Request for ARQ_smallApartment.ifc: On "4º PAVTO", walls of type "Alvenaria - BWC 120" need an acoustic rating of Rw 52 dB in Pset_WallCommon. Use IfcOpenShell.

First a look at what the model holds.

```python
import ifcopenshell
import ifcopenshell.util.element

model = ifcopenshell.open("ARQ_smallApartment.ifc")
print(model.schema)
storey = next(s for s in model.by_type("IfcBuildingStorey") if s.Name == "4º PAVTO")
walls = [e for e in ifcopenshell.util.element.get_decomposition(storey) if e.is_a("IfcWall")]
seen = {}
for e in walls:
    element_type = ifcopenshell.util.element.get_type(e)
    key = (element_type.Name if element_type != e and element_type else None, ifcopenshell.util.element.get_pset(e, "Pset_WallCommon", "AcousticRating"))
    seen[key] = seen.get(key, 0) + 1
for (name, value), count in sorted(seen.items(), key=str):
    print(count, "x", name, "|", value)
```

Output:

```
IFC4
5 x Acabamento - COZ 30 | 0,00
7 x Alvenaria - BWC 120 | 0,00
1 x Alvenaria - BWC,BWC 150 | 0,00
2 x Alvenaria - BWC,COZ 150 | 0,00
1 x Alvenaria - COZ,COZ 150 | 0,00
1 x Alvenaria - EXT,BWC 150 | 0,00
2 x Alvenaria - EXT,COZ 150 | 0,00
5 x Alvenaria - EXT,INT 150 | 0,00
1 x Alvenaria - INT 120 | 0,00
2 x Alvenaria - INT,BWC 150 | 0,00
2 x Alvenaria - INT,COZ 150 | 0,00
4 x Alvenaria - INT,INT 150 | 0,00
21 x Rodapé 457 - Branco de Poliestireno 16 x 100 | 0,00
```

```python
import ifcopenshell
import ifcopenshell.api.pset
import ifcopenshell.util.element

model = ifcopenshell.open("ARQ_smallApartment.ifc")

storey = next(s for s in model.by_type("IfcBuildingStorey") if s.Name == "4º PAVTO")
walls = [e for e in ifcopenshell.util.element.get_decomposition(storey) if e.is_a("IfcWall")]

count = 0
for e in walls:
    element_type = ifcopenshell.util.element.get_type(e)
    if element_type in (None, e) or element_type.Name != "Alvenaria - BWC 120":
        continue
    # add_pset returns the element's existing set when there is one.
    pset = ifcopenshell.api.pset.add_pset(model, product=e, name="Pset_WallCommon")
    ifcopenshell.api.pset.edit_pset(model, pset=pset, properties={"AcousticRating": "Rw 52 dB"})
    count += 1

print(count, "walls updated")

model.write("ARQ_smallApartment_v2.ifc")
```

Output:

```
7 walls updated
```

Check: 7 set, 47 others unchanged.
